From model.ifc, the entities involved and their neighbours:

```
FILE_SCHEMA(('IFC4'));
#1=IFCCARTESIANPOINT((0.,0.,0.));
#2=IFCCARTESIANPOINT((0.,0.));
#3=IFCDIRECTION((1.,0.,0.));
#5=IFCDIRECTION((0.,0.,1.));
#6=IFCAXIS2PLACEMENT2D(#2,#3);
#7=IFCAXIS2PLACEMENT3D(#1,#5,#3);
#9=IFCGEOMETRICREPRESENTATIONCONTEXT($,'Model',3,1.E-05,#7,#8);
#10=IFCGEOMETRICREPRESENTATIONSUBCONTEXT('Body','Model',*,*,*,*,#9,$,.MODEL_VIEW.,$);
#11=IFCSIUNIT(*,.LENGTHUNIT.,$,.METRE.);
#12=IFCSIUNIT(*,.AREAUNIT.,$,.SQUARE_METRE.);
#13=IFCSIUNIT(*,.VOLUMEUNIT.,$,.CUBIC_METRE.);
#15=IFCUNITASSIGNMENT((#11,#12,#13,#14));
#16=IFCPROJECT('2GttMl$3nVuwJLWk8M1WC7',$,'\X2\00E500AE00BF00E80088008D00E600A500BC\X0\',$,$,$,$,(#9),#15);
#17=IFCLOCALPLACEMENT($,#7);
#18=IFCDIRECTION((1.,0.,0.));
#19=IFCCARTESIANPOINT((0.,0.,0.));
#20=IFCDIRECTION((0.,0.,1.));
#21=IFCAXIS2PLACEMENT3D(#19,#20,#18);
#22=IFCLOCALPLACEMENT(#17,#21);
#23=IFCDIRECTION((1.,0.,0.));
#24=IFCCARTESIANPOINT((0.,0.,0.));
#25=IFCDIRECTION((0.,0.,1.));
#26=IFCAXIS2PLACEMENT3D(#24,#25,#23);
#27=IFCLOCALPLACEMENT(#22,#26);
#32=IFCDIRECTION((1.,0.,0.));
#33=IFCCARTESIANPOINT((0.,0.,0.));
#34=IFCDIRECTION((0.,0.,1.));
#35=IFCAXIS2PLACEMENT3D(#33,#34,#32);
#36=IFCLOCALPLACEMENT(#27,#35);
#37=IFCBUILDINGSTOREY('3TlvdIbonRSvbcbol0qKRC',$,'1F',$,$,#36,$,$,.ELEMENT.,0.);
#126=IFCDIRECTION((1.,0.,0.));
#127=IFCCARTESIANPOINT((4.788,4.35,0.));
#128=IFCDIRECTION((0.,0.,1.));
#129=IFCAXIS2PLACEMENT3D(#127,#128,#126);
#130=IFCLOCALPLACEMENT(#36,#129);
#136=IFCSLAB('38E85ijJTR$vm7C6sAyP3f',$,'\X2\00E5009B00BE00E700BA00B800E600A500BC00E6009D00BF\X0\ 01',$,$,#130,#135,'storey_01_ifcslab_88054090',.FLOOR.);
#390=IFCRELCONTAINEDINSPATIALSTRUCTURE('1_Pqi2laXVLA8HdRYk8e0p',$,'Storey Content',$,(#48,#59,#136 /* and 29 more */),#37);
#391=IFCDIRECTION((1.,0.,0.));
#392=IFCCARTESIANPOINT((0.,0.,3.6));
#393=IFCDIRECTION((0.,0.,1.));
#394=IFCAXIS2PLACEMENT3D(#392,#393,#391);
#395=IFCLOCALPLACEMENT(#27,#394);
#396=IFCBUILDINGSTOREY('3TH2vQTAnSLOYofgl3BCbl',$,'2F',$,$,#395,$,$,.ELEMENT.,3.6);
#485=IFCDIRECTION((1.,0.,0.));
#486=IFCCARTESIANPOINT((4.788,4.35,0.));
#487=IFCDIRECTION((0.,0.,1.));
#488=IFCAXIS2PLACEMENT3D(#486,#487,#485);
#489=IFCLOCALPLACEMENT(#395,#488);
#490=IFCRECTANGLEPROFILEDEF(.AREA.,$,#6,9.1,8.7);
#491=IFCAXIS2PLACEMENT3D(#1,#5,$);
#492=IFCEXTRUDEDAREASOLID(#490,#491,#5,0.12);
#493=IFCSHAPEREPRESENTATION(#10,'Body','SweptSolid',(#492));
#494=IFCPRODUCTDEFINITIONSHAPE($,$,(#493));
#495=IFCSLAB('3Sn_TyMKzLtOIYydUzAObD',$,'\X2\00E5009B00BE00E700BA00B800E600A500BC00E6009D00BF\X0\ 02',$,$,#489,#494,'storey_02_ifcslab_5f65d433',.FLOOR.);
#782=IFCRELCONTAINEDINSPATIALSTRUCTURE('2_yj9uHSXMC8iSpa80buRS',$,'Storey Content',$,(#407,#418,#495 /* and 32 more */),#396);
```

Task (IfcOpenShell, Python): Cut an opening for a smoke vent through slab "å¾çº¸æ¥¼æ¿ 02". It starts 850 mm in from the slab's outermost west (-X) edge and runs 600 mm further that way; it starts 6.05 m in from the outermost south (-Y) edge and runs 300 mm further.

```python
import numpy as np
import ifcopenshell
import ifcopenshell.api.feature
import ifcopenshell.api.geometry
import ifcopenshell.api.root
import ifcopenshell.geom
import ifcopenshell.util.placement
import ifcopenshell.util.representation
import ifcopenshell.util.shape
import ifcopenshell.util.unit

model = ifcopenshell.open("model.ifc")
unit_scale = ifcopenshell.util.unit.calculate_unit_scale(model)
settings = ifcopenshell.geom.settings()


def volume(element):
    """Net volume in cubic metres, openings subtracted."""
    shape = ifcopenshell.geom.create_shape(settings, element)
    return ifcopenshell.util.shape.get_volume(shape.geometry)


slab = model.by_id(495)
before = volume(slab)

# Extent in the slab's own axes, in metres. The edges named are its -X and -Y sides.
slab_shape = ifcopenshell.geom.create_shape(settings, slab)
vertices = ifcopenshell.util.shape.get_vertices(slab_shape.geometry)
x_min, y_min, bottom = vertices.min(axis=0)
top = vertices[:, 2].max()

opening = ifcopenshell.api.root.create_entity(model, ifc_class="IfcOpeningElement", name="Smoke vent opening", predefined_type="OPENING")
context = ifcopenshell.util.representation.get_context(model, "Model", "Body", "MODEL_VIEW")
width, depth = 0.6, 0.3
outline = [(0.0, 0.0), (width, 0.0), (width, depth), (0.0, depth), (0.0, 0.0)]
# Overshoot both faces by 50 mm so the cut is clean.
shape = ifcopenshell.api.geometry.add_slab_representation(
    model, context=context, depth=top - bottom + 0.1, polyline=outline
)
ifcopenshell.api.geometry.assign_representation(model, product=opening, representation=shape)

matrix = ifcopenshell.util.placement.get_local_placement(slab.ObjectPlacement)
matrix[:, 3] = matrix @ np.append(np.array([x_min + 0.85, y_min + 6.05, bottom - 0.05]) / unit_scale, 1.0)
ifcopenshell.api.geometry.edit_object_placement(model, product=opening, matrix=matrix, is_si=False)
ifcopenshell.api.feature.add_feature(model, feature=opening, element=slab)

after = volume(slab)

print(f"slab volume {before:.3f} -> {after:.3f} m3")

model.write("model-out.ifc")
```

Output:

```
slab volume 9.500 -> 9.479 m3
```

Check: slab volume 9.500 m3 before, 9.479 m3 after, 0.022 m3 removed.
